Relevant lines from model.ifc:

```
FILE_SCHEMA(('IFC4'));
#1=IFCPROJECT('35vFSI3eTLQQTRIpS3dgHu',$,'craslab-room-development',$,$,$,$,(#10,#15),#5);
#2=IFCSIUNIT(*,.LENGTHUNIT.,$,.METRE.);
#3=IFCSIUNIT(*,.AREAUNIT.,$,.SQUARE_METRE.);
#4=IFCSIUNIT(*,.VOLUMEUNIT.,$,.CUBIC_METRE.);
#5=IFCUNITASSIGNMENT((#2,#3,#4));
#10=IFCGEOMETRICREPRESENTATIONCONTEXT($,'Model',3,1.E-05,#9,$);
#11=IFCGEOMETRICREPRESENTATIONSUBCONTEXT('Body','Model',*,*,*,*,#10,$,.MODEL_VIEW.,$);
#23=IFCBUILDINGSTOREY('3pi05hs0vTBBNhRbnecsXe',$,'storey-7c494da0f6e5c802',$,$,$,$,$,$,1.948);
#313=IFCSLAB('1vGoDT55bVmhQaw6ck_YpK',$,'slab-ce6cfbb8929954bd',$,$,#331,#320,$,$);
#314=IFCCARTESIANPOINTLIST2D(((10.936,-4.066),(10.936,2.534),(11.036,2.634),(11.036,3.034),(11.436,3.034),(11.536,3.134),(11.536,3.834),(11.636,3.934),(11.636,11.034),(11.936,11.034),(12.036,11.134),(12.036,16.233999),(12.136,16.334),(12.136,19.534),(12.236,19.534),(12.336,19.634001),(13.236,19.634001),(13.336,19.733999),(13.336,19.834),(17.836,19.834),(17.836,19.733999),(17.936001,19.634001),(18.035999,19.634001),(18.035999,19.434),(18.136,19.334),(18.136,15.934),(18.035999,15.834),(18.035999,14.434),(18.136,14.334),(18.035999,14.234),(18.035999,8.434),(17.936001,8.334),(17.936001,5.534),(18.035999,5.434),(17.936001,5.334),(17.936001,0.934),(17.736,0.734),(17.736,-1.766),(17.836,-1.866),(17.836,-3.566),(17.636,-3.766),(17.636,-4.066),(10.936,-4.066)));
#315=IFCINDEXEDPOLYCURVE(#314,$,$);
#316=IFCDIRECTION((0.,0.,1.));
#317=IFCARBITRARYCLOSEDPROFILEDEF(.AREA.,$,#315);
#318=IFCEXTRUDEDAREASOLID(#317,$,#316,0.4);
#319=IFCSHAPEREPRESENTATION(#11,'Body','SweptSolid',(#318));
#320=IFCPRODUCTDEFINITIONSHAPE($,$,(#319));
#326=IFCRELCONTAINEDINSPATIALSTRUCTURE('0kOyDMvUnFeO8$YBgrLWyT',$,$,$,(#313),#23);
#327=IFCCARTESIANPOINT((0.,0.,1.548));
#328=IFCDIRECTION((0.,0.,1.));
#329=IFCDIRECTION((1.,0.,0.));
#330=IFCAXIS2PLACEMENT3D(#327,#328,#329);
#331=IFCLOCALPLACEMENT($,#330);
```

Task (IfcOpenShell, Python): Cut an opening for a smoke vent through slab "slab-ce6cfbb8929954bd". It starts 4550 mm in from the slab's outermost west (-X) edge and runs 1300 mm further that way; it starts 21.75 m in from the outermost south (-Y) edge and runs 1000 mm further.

```python
import numpy as np
import ifcopenshell
import ifcopenshell.api.feature
import ifcopenshell.api.geometry
import ifcopenshell.api.root
import ifcopenshell.geom
import ifcopenshell.util.placement
import ifcopenshell.util.representation
import ifcopenshell.util.shape
import ifcopenshell.util.unit

model = ifcopenshell.open("model.ifc")
unit_scale = ifcopenshell.util.unit.calculate_unit_scale(model)
settings = ifcopenshell.geom.settings()


def volume(element):
    """Net volume in cubic metres, openings subtracted."""
    shape = ifcopenshell.geom.create_shape(settings, element)
    return ifcopenshell.util.shape.get_volume(shape.geometry)


slab = model.by_id(313)
before = volume(slab)

# Extent in the slab's own axes, in metres. The edges named are its -X and -Y sides.
slab_shape = ifcopenshell.geom.create_shape(settings, slab)
vertices = ifcopenshell.util.shape.get_vertices(slab_shape.geometry)
x_min, y_min, bottom = vertices.min(axis=0)
top = vertices[:, 2].max()

opening = ifcopenshell.api.root.create_entity(model, ifc_class="IfcOpeningElement", name="Smoke vent opening", predefined_type="OPENING")
context = ifcopenshell.util.representation.get_context(model, "Model", "Body", "MODEL_VIEW")
width, depth = 1.3, 1
outline = [(0.0, 0.0), (width, 0.0), (width, depth), (0.0, depth), (0.0, 0.0)]
# Overshoot both faces by 50 mm so the cut is clean.
shape = ifcopenshell.api.geometry.add_slab_representation(
    model, context=context, depth=top - bottom + 0.1, polyline=outline
)
ifcopenshell.api.geometry.assign_representation(model, product=opening, representation=shape)

matrix = ifcopenshell.util.placement.get_local_placement(slab.ObjectPlacement)
matrix[:, 3] = matrix @ np.append(np.array([x_min + 4.55, y_min + 21.75, bottom - 0.05]) / unit_scale, 1.0)
ifcopenshell.api.geometry.edit_object_placement(model, product=opening, matrix=matrix, is_si=False)
ifcopenshell.api.feature.add_feature(model, feature=opening, element=slab)

after = volume(slab)

print(f"slab volume {before:.3f} -> {after:.3f} m3")

model.write("model-out.ifc")
```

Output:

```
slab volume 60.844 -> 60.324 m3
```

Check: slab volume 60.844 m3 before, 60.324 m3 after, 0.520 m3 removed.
